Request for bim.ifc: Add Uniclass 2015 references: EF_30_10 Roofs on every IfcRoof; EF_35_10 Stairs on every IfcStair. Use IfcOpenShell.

First a look at what the model holds.

```python
import ifcopenshell

model = ifcopenshell.open("bim.ifc")
print(model.schema)
print("classifications:", [c.Name for c in model.by_type("IfcClassification")])
for ifc_class in ("IfcDoor", "IfcRoof", "IfcStair", "IfcWall", "IfcWindow"):
    print(ifc_class, len(model.by_type(ifc_class)))
```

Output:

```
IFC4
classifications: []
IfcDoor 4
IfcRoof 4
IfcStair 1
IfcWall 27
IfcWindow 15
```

```python
import ifcopenshell
import ifcopenshell.api.classification

model = ifcopenshell.open("bim.ifc")

system = ifcopenshell.api.classification.add_classification(model, classification="Uniclass 2015")

codes = {
    "IfcRoof": ("EF_30_10", "Roofs"),
    "IfcStair": ("EF_35_10", "Stairs"),
}
for ifc_class, (code, name) in codes.items():
    products = model.by_type(ifc_class)
    ifcopenshell.api.classification.add_reference(
        model, products=products, classification=system, identification=code, name=name
    )
    print(code, len(products))

model.write("bim_v2.ifc")
```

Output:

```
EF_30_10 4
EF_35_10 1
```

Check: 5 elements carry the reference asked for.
